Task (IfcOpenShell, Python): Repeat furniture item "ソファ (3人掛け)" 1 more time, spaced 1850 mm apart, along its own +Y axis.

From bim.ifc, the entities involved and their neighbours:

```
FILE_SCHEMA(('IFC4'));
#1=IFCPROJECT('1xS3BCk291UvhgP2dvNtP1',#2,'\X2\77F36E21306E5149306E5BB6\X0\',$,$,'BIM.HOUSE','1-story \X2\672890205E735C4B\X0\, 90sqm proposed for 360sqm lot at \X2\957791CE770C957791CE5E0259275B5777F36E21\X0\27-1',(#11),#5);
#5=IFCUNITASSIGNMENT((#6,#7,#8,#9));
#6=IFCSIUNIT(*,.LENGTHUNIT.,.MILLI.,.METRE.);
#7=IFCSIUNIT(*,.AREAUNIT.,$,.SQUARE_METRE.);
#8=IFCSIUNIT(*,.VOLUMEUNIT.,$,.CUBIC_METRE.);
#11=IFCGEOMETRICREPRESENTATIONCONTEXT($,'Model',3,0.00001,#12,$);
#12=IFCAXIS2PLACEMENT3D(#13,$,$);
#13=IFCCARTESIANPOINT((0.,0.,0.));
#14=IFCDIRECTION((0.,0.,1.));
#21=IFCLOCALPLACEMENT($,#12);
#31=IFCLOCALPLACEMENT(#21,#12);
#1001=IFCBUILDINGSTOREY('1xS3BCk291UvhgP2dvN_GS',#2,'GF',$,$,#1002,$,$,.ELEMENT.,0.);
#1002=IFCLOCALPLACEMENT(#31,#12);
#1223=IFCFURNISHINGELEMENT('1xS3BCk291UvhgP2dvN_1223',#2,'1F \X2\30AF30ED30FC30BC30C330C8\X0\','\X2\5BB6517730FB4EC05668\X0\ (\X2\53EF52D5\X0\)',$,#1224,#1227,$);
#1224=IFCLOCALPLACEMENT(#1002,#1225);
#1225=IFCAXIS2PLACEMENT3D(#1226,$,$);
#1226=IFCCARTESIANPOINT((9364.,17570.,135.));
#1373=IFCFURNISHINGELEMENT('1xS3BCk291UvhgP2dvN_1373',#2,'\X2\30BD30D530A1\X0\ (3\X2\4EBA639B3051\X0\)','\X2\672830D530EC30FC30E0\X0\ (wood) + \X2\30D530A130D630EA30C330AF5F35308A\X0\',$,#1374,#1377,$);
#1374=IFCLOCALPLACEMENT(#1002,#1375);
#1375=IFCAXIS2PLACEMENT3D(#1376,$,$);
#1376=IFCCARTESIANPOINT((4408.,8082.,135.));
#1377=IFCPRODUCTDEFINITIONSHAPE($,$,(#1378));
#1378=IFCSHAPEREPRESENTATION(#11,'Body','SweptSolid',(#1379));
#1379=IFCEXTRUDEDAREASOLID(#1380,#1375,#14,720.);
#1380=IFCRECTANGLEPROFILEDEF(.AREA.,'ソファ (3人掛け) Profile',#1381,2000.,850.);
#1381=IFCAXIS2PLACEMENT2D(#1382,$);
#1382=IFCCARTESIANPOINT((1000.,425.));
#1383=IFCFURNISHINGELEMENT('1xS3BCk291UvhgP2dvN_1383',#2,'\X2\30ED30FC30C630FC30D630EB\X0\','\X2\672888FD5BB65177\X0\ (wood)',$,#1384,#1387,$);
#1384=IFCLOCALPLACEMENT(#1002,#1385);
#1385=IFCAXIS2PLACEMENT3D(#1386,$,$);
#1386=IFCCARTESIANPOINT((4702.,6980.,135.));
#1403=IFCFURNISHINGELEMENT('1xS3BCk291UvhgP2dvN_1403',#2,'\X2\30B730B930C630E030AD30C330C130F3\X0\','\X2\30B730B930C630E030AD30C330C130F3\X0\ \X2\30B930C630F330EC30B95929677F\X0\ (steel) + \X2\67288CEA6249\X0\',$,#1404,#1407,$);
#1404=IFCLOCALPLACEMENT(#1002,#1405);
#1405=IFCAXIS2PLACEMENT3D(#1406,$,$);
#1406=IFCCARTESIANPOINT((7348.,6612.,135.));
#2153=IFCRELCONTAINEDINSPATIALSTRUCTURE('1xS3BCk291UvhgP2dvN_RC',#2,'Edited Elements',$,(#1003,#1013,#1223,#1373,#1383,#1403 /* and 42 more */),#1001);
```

```python
import ifcopenshell
import ifcopenshell.api.geometry
import ifcopenshell.api.root
import ifcopenshell.util.element
import ifcopenshell.util.placement
import ifcopenshell.util.unit

model = ifcopenshell.open("bim.ifc")
unit_scale = ifcopenshell.util.unit.calculate_unit_scale(model)


def reuse_history(source, copy):
    """copy_class also copies each property set's owner history, people and application; keep the originals."""
    for rel in copy.IsDefinedBy:
        if rel.is_a("IfcRelDefinesByProperties") and (history := rel.RelatingPropertyDefinition.OwnerHistory):
            rel.RelatingPropertyDefinition.OwnerHistory = source.OwnerHistory
            ifcopenshell.util.element.remove_deep2(model, history)


source = model.by_id(1373)
base = ifcopenshell.util.placement.get_local_placement(source.ObjectPlacement)
step = base[:3, 1] * 1.85 / unit_scale

for i in range(1, 2):
    copy = ifcopenshell.api.root.copy_class(model, product=source)
    copy.Representation = ifcopenshell.util.element.copy_deep(
        model, source.Representation, exclude=["IfcGeometricRepresentationContext", "IfcRepresentationMap"]
    )
    reuse_history(source, copy)
    matrix = base.copy()
    matrix[:3, 3] += i * step
    print("added at", matrix[:3, 3].round(3) + 0.0)
    ifcopenshell.api.geometry.edit_object_placement(model, product=copy, matrix=matrix, is_si=False)

model.write("bim-out.ifc")
```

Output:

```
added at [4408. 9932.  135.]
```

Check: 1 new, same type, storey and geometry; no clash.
